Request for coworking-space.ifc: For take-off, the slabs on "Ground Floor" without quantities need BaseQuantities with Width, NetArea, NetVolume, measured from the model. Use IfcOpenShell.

First a look at what the model holds.

```python
import ifcopenshell
import ifcopenshell.util.element
import ifcopenshell.util.unit

model = ifcopenshell.open("coworking-space.ifc")
print(model.schema)
for unit_type in ("LENGTHUNIT", "AREAUNIT", "VOLUMEUNIT"):
    print(unit_type, ifcopenshell.util.unit.calculate_unit_scale(model, unit_type))
storey = next(s for s in model.by_type("IfcBuildingStorey") if s.Name == "Ground Floor")
slabs = [e for e in ifcopenshell.util.element.get_decomposition(storey) if e.is_a("IfcSlab")]
for e in sorted(slabs, key=lambda e: e.id()):
    print(e.id(), e.is_a(), e.Name, list(ifcopenshell.util.element.get_psets(e, qtos_only=True)), sep=" | ")
```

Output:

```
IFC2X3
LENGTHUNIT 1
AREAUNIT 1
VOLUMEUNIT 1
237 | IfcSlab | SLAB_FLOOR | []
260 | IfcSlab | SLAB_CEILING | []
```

```python
import ifcopenshell
import ifcopenshell.api.pset
import ifcopenshell.geom
import ifcopenshell.util.element
import ifcopenshell.util.shape
import ifcopenshell.util.unit

model = ifcopenshell.open("coworking-space.ifc")
unit_scale = ifcopenshell.util.unit.calculate_unit_scale(model)
area_scale = ifcopenshell.util.unit.calculate_unit_scale(model, "AREAUNIT")
volume_scale = ifcopenshell.util.unit.calculate_unit_scale(model, "VOLUMEUNIT")
settings = ifcopenshell.geom.settings()

storey = next(s for s in model.by_type("IfcBuildingStorey") if s.Name == "Ground Floor")
slabs = [e for e in ifcopenshell.util.element.get_decomposition(storey) if e.is_a("IfcSlab")]

for e in sorted(slabs, key=lambda e: e.id()):
    if ifcopenshell.util.element.get_psets(e, qtos_only=True, should_inherit=False):
        continue
    # Geometry comes back in metres, in the element's own axes.
    shape = ifcopenshell.geom.create_shape(settings, e)
    values = {
        "Width": ifcopenshell.util.shape.get_z(shape.geometry) / unit_scale,
        "NetArea": ifcopenshell.util.shape.get_footprint_area(shape.geometry) / area_scale,
        "NetVolume": ifcopenshell.util.shape.get_volume(shape.geometry) / volume_scale,
    }
    qto = ifcopenshell.api.pset.add_qto(model, product=e, name="BaseQuantities")
    ifcopenshell.api.pset.edit_qto(model, qto=qto, properties=values)
    print(e.id(), {k: round(v, 3) for k, v in values.items()})

model.write("coworking-space_v2.ifc")
```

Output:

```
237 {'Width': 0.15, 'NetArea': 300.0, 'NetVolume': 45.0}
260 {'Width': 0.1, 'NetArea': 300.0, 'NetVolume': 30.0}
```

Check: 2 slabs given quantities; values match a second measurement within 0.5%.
